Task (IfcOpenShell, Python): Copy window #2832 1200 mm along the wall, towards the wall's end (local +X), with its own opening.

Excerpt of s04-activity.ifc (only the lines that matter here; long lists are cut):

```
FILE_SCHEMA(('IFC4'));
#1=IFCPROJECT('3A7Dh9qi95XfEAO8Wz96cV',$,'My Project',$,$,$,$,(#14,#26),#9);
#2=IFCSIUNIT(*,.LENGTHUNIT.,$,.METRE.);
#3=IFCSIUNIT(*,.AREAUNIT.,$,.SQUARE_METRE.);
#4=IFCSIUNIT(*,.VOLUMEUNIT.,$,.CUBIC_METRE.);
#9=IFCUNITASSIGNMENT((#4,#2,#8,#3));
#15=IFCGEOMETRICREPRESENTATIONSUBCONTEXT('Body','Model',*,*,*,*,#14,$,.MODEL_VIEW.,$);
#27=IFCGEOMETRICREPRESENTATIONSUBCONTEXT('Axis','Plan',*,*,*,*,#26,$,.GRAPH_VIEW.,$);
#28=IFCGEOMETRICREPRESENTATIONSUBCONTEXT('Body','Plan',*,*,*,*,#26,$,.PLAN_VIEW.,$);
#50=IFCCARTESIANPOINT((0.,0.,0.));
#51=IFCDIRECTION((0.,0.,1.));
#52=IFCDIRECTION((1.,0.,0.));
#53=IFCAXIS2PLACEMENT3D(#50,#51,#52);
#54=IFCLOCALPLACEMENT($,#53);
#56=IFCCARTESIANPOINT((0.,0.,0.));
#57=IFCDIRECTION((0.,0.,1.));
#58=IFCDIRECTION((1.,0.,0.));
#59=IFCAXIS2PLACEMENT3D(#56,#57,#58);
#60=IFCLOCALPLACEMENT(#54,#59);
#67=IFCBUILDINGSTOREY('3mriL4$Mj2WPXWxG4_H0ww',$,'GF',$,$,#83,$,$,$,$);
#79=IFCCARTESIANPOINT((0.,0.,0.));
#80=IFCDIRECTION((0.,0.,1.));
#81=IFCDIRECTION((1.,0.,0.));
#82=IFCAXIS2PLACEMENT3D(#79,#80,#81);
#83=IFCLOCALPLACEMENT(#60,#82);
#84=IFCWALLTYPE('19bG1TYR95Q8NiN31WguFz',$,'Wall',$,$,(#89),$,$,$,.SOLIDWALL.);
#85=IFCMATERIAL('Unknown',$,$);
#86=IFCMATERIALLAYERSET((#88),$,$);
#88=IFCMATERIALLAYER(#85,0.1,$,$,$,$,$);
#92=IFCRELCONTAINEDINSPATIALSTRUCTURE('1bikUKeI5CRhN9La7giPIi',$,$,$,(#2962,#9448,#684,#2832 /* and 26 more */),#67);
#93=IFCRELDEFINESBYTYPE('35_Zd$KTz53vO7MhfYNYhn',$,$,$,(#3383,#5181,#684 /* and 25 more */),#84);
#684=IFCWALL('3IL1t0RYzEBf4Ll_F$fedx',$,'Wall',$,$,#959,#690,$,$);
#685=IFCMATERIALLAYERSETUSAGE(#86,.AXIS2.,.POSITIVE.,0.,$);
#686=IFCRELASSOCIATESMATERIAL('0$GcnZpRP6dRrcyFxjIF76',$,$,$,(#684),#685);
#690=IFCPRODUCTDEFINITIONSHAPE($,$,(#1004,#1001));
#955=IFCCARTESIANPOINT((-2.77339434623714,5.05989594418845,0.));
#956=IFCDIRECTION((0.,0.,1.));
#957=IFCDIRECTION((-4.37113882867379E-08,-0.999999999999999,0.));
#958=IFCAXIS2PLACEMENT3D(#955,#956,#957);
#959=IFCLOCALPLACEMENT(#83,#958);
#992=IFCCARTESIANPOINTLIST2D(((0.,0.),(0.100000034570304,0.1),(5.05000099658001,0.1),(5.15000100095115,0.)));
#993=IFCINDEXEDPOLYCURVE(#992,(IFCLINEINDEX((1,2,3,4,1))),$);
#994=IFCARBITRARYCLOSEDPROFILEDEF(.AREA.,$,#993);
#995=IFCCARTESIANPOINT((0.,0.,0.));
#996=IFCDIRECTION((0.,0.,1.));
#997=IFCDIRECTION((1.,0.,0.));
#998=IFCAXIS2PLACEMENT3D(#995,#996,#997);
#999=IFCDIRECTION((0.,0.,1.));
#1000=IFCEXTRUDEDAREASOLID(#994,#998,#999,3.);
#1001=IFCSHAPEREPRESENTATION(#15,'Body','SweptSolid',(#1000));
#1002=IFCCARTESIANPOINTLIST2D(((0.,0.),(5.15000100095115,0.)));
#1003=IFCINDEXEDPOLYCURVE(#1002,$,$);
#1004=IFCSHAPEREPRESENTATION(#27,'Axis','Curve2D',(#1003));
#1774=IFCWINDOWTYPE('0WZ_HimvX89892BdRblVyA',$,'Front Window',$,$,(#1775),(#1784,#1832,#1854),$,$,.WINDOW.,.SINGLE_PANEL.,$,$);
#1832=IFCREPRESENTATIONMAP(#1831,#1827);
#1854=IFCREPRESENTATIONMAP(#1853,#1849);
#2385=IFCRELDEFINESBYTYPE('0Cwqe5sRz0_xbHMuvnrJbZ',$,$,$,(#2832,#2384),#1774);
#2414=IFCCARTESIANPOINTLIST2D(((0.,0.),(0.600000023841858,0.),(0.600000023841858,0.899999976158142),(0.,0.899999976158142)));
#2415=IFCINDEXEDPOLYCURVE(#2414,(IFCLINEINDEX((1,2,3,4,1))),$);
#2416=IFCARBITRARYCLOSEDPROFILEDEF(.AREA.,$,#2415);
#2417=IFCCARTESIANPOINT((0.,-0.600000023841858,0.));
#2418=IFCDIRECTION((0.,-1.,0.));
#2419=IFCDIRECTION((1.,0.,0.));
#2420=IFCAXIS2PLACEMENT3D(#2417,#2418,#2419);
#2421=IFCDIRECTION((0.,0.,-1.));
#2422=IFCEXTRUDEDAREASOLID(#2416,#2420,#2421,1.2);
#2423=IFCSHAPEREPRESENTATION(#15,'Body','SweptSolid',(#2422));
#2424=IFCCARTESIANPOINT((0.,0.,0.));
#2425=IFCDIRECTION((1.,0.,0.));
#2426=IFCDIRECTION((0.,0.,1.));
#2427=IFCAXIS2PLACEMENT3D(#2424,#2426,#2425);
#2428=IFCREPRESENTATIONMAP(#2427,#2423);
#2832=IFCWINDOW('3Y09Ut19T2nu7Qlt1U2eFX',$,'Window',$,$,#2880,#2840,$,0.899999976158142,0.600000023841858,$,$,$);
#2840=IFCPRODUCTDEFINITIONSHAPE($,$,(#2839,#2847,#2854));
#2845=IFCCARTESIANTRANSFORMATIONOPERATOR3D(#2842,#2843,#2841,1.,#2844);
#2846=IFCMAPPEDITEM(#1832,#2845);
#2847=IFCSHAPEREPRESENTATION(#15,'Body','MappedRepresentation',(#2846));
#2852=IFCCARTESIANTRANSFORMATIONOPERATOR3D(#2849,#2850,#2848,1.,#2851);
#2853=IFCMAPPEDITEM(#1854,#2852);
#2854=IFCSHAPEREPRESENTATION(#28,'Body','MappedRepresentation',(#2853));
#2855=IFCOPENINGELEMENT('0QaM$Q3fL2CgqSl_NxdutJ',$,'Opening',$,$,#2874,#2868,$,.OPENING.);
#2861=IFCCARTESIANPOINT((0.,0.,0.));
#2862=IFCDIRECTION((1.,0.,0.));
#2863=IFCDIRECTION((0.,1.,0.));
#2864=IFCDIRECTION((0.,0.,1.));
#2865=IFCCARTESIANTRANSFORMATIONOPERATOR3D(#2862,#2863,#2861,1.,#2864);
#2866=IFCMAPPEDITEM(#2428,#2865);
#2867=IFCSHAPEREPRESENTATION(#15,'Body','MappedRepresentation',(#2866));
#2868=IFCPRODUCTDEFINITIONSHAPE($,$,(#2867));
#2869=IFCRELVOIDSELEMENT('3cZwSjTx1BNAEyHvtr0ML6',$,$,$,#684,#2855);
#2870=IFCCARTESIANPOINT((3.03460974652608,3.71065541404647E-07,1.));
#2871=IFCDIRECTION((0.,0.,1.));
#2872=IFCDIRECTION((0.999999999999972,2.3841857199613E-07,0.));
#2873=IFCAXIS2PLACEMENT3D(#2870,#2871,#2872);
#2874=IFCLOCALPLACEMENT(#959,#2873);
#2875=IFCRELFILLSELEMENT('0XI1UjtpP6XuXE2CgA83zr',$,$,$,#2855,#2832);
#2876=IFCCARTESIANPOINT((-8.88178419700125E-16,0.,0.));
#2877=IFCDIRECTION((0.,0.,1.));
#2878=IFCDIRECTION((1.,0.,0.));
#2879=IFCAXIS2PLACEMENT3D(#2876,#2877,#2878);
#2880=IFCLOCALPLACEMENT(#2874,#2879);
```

```python
import ifcopenshell
import ifcopenshell.api.feature
import ifcopenshell.api.geometry
import ifcopenshell.api.root
import ifcopenshell.geom
import ifcopenshell.util.element
import ifcopenshell.util.placement
import ifcopenshell.util.shape
import ifcopenshell.util.unit

model = ifcopenshell.open("s04-activity.ifc")
unit_scale = ifcopenshell.util.unit.calculate_unit_scale(model)
settings = ifcopenshell.geom.settings()


def volume(element):
    """Net volume in cubic metres, openings subtracted."""
    shape = ifcopenshell.geom.create_shape(settings, element)
    return ifcopenshell.util.shape.get_volume(shape.geometry)


window = model.by_guid("3Y09Ut19T2nu7Qlt1U2eFX")
opening = window.FillsVoids[0].RelatingOpeningElement
wall = opening.VoidsElements[0].RelatingBuildingElement
before = volume(wall)
shift = ifcopenshell.util.placement.get_local_placement(wall.ObjectPlacement)[:3, 0] * 1.2 / unit_scale

# copy_class copies the void relationship, type, container and properties, but no geometry.
new_opening = ifcopenshell.api.root.copy_class(model, product=opening)
new_opening.Representation = ifcopenshell.util.element.copy_deep(
    model, opening.Representation, exclude=["IfcGeometricRepresentationContext", "IfcRepresentationMap"]
)
new_window = ifcopenshell.api.root.copy_class(model, product=window)
new_window.Representation = ifcopenshell.util.element.copy_deep(
    model, window.Representation, exclude=["IfcGeometricRepresentationContext", "IfcRepresentationMap"]
)
ifcopenshell.api.feature.add_filling(model, opening=new_opening, element=new_window)

for old, new in ((opening, new_opening), (window, new_window)):
    matrix = ifcopenshell.util.placement.get_local_placement(old.ObjectPlacement)
    matrix[:3, 3] += shift
    ifcopenshell.api.geometry.edit_object_placement(model, product=new, matrix=matrix, is_si=False)

after = volume(wall)

print(f"wall volume {before:.3f} -> {after:.3f} m3")

model.write("s04-activity_rev.ifc")
```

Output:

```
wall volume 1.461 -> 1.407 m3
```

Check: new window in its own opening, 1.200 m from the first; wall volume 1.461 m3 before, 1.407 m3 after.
